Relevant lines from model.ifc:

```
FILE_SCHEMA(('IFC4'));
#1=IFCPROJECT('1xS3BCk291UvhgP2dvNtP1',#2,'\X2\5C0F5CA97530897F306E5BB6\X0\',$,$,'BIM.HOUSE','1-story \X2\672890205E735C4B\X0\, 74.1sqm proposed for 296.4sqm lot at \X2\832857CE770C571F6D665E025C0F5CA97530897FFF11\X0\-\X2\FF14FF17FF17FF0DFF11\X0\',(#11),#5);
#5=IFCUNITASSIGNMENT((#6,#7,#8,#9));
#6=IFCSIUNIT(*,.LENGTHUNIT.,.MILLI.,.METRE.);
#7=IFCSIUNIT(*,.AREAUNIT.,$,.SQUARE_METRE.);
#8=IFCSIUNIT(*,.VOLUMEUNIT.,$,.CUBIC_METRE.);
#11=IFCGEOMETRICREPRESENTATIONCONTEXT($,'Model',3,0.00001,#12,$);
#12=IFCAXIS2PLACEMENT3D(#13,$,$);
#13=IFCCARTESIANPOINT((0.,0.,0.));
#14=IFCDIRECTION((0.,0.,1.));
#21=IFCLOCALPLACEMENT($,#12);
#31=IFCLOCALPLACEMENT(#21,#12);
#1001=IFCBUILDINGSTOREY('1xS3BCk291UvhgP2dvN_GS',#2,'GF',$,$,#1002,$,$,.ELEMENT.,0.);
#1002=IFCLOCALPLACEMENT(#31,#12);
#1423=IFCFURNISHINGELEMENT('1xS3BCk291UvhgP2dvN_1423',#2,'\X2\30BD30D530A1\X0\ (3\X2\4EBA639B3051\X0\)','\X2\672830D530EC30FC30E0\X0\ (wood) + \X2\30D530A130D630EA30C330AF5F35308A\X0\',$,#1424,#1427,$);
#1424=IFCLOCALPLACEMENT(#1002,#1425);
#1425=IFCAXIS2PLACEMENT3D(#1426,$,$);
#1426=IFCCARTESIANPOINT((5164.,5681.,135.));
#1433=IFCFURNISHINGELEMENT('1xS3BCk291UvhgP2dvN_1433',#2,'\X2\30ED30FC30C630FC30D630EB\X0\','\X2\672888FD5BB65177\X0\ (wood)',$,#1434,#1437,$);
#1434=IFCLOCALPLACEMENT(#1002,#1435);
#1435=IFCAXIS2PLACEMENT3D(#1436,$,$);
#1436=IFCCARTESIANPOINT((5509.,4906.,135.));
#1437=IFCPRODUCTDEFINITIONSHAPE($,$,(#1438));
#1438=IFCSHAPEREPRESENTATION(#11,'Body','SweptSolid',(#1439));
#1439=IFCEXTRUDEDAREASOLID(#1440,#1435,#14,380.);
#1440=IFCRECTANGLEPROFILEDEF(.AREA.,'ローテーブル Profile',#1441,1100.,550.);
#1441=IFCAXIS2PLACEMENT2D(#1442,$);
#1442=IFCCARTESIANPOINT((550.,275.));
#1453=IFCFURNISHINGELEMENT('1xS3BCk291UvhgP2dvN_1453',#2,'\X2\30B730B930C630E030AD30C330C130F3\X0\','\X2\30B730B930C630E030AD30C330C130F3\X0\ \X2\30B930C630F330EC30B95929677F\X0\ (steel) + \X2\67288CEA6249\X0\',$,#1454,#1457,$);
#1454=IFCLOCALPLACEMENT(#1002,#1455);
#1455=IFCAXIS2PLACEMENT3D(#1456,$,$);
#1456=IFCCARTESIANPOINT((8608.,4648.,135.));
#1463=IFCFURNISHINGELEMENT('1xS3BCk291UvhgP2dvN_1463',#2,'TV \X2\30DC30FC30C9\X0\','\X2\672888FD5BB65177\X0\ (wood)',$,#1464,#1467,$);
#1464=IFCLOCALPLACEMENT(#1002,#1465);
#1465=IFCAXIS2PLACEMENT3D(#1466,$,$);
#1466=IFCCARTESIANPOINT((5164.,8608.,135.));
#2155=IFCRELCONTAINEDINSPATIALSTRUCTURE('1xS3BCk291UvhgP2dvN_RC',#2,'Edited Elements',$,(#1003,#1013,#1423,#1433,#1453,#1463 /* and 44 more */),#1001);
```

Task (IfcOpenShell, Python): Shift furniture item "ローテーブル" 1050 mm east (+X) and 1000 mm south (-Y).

```python
import ifcopenshell
import ifcopenshell.api.geometry
import ifcopenshell.util.placement
import ifcopenshell.util.unit

model = ifcopenshell.open("model.ifc")
unit_scale = ifcopenshell.util.unit.calculate_unit_scale(model)

item = model.by_guid("1xS3BCk291UvhgP2dvN_1433")
matrix = ifcopenshell.util.placement.get_local_placement(item.ObjectPlacement)
matrix[0, 3] += 1.05 / unit_scale
matrix[1, 3] -= 1 / unit_scale
ifcopenshell.api.geometry.edit_object_placement(model, product=item, matrix=matrix, is_si=False)

print(ifcopenshell.util.placement.get_local_placement(item.ObjectPlacement).round(3) + 0.0)

model.write("model-out.ifc")
```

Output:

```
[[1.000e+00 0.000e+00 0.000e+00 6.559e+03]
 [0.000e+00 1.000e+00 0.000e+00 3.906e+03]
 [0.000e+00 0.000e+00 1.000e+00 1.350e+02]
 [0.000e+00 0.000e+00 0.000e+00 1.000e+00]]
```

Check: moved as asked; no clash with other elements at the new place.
